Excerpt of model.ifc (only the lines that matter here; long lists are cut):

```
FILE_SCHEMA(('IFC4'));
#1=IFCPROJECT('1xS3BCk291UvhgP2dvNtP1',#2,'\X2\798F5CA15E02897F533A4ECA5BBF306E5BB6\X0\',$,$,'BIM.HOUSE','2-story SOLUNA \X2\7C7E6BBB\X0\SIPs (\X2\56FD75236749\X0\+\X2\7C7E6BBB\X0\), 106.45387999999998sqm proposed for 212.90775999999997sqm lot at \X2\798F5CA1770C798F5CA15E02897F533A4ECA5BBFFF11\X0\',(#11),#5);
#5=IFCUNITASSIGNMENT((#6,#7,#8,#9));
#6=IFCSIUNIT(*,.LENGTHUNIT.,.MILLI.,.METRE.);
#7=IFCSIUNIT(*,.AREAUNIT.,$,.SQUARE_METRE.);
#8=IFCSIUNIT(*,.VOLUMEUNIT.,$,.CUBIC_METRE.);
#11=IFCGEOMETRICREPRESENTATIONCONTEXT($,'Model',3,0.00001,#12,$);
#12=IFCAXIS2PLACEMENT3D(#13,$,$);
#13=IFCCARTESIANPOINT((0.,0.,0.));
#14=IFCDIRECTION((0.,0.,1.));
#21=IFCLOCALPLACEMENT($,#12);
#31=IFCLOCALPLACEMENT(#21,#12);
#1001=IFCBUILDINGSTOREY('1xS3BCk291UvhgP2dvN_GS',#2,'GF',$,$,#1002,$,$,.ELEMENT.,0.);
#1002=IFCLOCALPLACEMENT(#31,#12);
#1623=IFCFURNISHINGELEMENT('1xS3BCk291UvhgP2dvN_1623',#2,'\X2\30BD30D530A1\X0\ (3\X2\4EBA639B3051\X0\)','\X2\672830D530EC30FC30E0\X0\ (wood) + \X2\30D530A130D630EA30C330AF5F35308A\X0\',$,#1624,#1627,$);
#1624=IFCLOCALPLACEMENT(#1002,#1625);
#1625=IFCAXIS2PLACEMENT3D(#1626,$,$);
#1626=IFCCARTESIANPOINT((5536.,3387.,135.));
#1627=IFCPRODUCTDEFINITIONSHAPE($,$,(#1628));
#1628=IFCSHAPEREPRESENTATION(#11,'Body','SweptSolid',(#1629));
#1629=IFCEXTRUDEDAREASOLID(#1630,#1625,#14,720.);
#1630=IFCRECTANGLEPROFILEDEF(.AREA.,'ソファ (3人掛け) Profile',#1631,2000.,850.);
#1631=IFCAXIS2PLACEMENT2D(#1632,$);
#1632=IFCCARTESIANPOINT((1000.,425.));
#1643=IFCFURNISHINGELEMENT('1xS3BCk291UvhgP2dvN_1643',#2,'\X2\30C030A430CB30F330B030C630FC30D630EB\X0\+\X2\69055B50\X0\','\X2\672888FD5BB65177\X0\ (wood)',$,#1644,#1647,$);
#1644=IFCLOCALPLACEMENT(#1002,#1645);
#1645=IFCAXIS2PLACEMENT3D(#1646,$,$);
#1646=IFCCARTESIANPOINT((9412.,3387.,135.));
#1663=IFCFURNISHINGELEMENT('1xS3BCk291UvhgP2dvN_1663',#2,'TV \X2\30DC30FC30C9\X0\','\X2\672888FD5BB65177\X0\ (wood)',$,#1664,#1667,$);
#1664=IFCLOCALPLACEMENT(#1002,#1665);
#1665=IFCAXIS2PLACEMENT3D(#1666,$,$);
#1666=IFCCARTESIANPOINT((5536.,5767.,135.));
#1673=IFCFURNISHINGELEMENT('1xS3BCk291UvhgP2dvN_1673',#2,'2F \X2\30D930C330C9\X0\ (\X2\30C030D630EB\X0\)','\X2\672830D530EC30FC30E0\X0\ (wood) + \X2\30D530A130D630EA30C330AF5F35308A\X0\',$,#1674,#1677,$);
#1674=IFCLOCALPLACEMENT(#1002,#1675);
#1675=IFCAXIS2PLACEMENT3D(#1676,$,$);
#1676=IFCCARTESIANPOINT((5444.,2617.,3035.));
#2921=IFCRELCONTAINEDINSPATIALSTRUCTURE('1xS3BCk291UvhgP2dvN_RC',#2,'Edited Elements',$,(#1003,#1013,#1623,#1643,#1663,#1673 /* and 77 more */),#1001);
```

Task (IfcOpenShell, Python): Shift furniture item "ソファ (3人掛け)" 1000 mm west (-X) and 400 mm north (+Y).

```python
import ifcopenshell
import ifcopenshell.api.geometry
import ifcopenshell.util.placement

model = ifcopenshell.open("model.ifc")

item = model.by_guid("1xS3BCk291UvhgP2dvN_1623")
matrix = ifcopenshell.util.placement.get_local_placement(item.ObjectPlacement)
matrix[0, 3] -= 1000.0
matrix[1, 3] += 400.0
ifcopenshell.api.geometry.edit_object_placement(model, product=item, matrix=matrix, is_si=False)

print(ifcopenshell.util.placement.get_local_placement(item.ObjectPlacement).round(3) + 0.0)

model.write("model_rev.ifc")
```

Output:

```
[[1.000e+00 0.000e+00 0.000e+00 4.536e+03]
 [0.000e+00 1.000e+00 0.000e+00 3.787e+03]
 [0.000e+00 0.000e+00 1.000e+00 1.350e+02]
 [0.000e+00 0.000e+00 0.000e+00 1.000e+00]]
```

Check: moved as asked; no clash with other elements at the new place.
